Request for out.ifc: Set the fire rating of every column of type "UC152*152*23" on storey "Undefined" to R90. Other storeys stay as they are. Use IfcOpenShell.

First a look at what the model holds.

```python
import ifcopenshell
import ifcopenshell.util.element

model = ifcopenshell.open("out.ifc")
print(model.schema)
storey = next(s for s in model.by_type("IfcBuildingStorey") if s.Name == "Undefined")
columns = [e for e in ifcopenshell.util.element.get_decomposition(storey) if e.is_a("IfcColumn")]
seen = {}
for e in columns:
    element_type = ifcopenshell.util.element.get_type(e)
    key = (element_type.Name if element_type != e and element_type else None, ifcopenshell.util.element.get_pset(e, "Pset_ColumnCommon", "FireRating"))
    seen[key] = seen.get(key, 0) + 1
for (name, value), count in sorted(seen.items(), key=str):
    print(count, "x", name, "|", value)
```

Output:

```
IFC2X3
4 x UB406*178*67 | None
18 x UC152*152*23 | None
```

```python
import ifcopenshell
import ifcopenshell.api.pset
import ifcopenshell.util.element

model = ifcopenshell.open("out.ifc")

storey = next(s for s in model.by_type("IfcBuildingStorey") if s.Name == "Undefined")
columns = [e for e in ifcopenshell.util.element.get_decomposition(storey) if e.is_a("IfcColumn")]

count = 0
for e in columns:
    element_type = ifcopenshell.util.element.get_type(e)
    if element_type in (None, e) or element_type.Name != "UC152*152*23":
        continue
    found = ifcopenshell.util.element.get_pset(e, "Pset_ColumnCommon", should_inherit=False)
    if found:
        pset = model.by_id(found["id"])
        if len(ifcopenshell.util.element.get_elements_by_pset(pset)) > 1:
            pset = ifcopenshell.api.pset.unshare_pset(model, products=[e], pset=pset)[0]
    else:
        pset = ifcopenshell.api.pset.add_pset(model, product=e, name="Pset_ColumnCommon")
    ifcopenshell.api.pset.edit_pset(model, pset=pset, properties={"FireRating": "R90"})
    count += 1

print(count, "columns updated")

model.write("out_updated.ifc")
```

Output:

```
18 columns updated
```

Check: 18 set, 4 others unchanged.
